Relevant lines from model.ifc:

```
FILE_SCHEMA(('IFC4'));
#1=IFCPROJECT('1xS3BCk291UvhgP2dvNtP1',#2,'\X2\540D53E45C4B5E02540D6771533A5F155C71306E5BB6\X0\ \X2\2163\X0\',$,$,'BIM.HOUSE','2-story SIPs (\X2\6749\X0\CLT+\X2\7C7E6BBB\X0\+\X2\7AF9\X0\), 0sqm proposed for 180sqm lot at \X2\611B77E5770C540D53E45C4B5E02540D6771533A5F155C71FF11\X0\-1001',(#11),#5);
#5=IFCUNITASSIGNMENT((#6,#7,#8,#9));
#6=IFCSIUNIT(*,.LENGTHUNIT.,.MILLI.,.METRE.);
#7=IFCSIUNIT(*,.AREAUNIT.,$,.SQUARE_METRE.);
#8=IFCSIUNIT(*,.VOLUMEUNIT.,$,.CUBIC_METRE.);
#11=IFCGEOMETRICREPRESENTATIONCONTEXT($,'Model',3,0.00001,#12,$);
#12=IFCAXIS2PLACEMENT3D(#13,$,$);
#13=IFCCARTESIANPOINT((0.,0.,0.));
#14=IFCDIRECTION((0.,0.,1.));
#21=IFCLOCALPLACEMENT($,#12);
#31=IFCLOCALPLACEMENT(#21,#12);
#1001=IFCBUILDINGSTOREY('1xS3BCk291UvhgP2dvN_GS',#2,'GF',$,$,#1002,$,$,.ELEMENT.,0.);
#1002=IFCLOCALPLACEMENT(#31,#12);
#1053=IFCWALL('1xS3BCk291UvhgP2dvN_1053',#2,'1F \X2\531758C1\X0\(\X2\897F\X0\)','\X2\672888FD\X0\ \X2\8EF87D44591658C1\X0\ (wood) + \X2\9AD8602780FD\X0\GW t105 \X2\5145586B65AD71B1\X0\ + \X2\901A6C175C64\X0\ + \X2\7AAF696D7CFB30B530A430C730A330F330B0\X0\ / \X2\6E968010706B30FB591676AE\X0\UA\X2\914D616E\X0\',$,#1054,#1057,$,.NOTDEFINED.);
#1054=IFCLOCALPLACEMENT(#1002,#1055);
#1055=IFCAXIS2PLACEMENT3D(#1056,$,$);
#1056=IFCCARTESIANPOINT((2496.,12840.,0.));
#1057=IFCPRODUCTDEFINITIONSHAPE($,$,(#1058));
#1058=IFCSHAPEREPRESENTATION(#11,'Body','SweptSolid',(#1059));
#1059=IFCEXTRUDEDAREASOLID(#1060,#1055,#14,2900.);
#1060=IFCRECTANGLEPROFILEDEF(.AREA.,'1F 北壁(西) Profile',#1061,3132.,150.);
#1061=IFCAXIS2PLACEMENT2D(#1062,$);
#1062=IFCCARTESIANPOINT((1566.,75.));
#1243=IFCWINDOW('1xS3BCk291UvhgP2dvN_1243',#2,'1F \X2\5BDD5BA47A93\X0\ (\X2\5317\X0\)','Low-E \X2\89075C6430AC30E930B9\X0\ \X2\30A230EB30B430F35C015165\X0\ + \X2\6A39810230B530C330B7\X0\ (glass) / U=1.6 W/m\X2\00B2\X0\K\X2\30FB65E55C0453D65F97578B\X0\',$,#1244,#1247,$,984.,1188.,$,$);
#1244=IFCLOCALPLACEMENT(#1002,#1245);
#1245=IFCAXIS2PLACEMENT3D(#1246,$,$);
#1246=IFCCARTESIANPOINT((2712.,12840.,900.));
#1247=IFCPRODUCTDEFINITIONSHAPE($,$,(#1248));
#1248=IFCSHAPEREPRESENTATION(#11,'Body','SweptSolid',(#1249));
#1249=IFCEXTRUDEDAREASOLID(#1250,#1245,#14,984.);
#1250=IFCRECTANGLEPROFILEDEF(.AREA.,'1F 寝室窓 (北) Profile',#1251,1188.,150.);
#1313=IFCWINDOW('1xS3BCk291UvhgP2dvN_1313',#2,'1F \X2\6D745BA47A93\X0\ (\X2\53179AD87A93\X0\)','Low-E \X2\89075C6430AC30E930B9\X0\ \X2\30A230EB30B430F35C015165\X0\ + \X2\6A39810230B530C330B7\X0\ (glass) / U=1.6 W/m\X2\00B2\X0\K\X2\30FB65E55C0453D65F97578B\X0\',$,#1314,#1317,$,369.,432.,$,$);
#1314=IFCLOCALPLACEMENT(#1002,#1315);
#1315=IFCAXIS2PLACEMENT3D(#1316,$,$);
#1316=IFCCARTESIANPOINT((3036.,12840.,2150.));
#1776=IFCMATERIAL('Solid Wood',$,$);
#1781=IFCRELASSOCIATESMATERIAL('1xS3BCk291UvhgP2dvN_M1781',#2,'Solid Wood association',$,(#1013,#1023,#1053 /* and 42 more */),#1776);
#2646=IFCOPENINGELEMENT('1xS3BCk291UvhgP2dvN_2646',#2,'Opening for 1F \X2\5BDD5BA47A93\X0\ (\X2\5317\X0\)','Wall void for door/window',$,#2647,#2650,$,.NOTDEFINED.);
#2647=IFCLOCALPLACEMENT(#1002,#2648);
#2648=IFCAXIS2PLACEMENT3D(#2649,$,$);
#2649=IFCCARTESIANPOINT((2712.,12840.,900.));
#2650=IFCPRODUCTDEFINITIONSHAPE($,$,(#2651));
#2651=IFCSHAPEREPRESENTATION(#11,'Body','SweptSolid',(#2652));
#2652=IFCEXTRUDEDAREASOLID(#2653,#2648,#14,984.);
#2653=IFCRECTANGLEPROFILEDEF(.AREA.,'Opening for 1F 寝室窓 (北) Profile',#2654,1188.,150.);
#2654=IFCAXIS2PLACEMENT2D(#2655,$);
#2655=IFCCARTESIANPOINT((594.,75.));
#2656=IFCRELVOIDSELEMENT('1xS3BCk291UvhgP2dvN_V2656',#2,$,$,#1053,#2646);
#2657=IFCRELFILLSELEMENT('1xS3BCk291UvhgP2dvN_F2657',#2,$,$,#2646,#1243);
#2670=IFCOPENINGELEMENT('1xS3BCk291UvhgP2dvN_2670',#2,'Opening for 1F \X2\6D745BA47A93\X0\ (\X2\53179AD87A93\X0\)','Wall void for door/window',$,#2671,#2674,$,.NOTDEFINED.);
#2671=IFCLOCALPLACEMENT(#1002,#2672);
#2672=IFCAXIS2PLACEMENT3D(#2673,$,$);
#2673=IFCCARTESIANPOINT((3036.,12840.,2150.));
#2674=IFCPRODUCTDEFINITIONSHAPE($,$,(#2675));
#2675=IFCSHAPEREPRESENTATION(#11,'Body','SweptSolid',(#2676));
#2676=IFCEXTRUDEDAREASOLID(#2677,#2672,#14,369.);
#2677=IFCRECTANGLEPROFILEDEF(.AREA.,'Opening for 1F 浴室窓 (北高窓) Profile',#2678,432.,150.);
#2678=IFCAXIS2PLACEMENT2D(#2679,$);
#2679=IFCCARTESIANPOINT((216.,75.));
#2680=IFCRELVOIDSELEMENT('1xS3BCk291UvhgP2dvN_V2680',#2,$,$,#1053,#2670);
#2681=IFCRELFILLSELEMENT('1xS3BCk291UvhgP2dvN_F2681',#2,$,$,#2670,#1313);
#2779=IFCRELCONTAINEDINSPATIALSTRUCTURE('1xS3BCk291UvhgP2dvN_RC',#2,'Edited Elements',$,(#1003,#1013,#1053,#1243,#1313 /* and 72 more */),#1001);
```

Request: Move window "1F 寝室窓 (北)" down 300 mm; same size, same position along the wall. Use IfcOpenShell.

```python
import numpy as np
import ifcopenshell
import ifcopenshell.api.geometry
import ifcopenshell.util.placement
import ifcopenshell.util.unit

model = ifcopenshell.open("model.ifc")
unit_scale = ifcopenshell.util.unit.calculate_unit_scale(model)

window = model.by_guid("1xS3BCk291UvhgP2dvN_1243")
opening = window.FillsVoids[0].RelatingOpeningElement
dz = -0.3 / unit_scale

shift = np.array([0.0, 0.0, dz])
# The window is not placed relative to its opening, so move both.
for product in (opening, window):
    matrix = ifcopenshell.util.placement.get_local_placement(product.ObjectPlacement)
    matrix[:3, 3] += shift
    ifcopenshell.api.geometry.edit_object_placement(model, product=product, matrix=matrix, is_si=False)

print(f"moved by {dz * unit_scale:+.3f} m")

model.write("model_rev.ifc")
```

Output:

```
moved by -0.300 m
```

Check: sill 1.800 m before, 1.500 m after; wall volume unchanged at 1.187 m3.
